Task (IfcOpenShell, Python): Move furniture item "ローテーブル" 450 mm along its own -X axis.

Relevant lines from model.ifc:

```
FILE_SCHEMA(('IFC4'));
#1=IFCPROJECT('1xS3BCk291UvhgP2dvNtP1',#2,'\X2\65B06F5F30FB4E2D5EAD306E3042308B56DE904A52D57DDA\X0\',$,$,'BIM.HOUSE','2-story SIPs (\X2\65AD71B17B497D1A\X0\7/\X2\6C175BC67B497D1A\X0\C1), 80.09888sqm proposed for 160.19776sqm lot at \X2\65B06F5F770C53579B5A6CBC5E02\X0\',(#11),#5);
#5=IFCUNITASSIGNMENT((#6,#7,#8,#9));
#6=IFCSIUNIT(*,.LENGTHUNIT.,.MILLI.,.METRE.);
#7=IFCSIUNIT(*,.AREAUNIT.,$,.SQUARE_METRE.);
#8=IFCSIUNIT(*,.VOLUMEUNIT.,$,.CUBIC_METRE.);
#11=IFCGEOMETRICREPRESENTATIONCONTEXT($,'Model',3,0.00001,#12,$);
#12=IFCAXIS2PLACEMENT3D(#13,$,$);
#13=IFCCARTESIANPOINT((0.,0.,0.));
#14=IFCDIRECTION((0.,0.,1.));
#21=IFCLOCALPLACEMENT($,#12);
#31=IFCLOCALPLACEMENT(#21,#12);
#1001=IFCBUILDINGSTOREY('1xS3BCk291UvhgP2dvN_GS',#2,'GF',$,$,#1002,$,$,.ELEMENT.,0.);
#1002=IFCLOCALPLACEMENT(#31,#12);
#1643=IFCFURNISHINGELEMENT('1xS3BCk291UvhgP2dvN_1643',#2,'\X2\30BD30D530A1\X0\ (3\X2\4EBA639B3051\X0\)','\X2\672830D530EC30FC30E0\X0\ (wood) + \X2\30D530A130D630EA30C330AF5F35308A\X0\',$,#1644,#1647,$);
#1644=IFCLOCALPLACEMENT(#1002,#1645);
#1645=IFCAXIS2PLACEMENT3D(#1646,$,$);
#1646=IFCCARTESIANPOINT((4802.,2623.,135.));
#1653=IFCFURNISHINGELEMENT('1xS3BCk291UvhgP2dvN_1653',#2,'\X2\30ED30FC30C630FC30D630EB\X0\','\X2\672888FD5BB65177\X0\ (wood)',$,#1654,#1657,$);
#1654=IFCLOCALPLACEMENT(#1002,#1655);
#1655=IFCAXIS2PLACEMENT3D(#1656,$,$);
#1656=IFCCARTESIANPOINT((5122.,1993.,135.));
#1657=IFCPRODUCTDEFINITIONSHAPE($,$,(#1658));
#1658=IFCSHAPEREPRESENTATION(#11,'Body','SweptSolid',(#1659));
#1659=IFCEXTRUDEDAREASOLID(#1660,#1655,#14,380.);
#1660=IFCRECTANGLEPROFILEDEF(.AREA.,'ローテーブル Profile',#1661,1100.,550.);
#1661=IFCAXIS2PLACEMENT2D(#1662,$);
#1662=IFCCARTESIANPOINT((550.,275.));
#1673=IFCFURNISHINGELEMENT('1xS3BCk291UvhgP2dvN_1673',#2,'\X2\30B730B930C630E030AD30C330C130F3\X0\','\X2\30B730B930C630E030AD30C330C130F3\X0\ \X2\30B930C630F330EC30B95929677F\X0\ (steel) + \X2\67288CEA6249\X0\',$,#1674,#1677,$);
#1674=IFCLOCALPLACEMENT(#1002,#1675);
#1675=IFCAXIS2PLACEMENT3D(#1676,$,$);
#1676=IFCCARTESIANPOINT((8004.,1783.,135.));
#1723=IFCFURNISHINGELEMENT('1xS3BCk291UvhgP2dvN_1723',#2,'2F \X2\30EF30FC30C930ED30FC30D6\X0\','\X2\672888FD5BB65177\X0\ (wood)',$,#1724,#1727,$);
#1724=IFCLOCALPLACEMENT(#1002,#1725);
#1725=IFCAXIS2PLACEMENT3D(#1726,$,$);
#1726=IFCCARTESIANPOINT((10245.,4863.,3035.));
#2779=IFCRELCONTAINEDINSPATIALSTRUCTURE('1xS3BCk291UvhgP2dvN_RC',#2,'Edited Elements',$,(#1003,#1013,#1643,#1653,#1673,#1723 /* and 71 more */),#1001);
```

```python
import ifcopenshell
import ifcopenshell.api.geometry
import ifcopenshell.util.placement
import ifcopenshell.util.unit

model = ifcopenshell.open("model.ifc")
unit_scale = ifcopenshell.util.unit.calculate_unit_scale(model)

item = model.by_guid("1xS3BCk291UvhgP2dvN_1653")
matrix = ifcopenshell.util.placement.get_local_placement(item.ObjectPlacement)
matrix[:3, 3] -= matrix[:3, 0] * 0.45 / unit_scale
ifcopenshell.api.geometry.edit_object_placement(model, product=item, matrix=matrix, is_si=False)

print(ifcopenshell.util.placement.get_local_placement(item.ObjectPlacement).round(3) + 0.0)

model.write("model_updated.ifc")
```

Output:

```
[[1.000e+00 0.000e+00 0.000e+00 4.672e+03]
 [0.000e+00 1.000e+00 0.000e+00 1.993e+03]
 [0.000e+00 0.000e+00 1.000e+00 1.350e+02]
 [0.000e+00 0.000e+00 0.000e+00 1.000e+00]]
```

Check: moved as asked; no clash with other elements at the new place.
